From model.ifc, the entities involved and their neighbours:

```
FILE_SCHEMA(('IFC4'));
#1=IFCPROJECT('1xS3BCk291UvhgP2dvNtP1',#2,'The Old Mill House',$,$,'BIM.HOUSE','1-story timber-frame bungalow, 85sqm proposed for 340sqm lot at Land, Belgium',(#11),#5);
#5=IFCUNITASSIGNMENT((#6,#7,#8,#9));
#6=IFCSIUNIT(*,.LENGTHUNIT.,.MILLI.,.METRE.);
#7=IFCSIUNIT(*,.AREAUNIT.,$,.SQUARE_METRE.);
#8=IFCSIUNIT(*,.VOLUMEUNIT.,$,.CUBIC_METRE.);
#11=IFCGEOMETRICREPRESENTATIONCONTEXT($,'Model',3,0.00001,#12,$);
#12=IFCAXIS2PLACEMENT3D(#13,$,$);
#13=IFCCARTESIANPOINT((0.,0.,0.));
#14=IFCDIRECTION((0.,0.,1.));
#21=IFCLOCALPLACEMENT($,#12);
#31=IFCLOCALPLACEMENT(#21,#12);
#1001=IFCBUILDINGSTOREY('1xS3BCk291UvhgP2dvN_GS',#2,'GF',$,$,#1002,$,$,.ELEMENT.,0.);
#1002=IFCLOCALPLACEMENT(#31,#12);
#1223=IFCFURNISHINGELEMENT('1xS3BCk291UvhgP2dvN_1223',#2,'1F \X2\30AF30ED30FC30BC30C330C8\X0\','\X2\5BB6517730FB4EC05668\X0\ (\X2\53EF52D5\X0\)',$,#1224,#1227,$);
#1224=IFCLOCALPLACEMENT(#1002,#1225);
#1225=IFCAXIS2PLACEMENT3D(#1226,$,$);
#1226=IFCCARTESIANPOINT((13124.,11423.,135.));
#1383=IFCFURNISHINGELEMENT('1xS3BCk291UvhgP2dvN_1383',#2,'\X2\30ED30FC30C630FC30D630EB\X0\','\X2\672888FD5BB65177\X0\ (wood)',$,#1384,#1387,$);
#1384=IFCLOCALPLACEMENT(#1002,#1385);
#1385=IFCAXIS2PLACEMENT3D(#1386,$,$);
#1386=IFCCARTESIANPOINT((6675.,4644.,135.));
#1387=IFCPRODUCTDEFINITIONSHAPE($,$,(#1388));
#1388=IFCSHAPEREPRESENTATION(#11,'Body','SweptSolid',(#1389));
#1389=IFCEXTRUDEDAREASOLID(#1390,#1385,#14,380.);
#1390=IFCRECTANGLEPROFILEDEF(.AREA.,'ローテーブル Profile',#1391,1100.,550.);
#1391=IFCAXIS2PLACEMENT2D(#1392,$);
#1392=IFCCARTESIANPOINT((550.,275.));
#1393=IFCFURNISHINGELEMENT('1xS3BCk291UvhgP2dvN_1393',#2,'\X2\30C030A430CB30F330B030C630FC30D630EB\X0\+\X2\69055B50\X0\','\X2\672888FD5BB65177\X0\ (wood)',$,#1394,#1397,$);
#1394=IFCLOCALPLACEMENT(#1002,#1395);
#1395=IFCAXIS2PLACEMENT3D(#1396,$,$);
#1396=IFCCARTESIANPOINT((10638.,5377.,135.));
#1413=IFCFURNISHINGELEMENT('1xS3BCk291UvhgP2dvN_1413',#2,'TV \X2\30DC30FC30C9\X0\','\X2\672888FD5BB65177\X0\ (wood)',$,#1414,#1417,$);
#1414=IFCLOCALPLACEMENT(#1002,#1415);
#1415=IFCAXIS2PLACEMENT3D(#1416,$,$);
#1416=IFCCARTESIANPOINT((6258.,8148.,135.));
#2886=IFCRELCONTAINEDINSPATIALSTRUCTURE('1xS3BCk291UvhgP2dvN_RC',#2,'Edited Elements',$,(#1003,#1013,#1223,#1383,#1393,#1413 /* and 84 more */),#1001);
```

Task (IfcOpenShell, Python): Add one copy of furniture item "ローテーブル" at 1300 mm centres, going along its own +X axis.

```python
import ifcopenshell
import ifcopenshell.api.geometry
import ifcopenshell.api.root
import ifcopenshell.util.element
import ifcopenshell.util.placement

model = ifcopenshell.open("model.ifc")


def reuse_history(source, copy):
    """copy_class also copies each property set's owner history, people and application; keep the originals."""
    for rel in copy.IsDefinedBy:
        if rel.is_a("IfcRelDefinesByProperties") and (history := rel.RelatingPropertyDefinition.OwnerHistory):
            rel.RelatingPropertyDefinition.OwnerHistory = source.OwnerHistory
            ifcopenshell.util.element.remove_deep2(model, history)


source = model.by_guid("1xS3BCk291UvhgP2dvN_1383")
base = ifcopenshell.util.placement.get_local_placement(source.ObjectPlacement)
step = base[:3, 0] * 1300.0

for i in range(1, 2):
    copy = ifcopenshell.api.root.copy_class(model, product=source)
    copy.Representation = ifcopenshell.util.element.copy_deep(
        model, source.Representation, exclude=["IfcGeometricRepresentationContext", "IfcRepresentationMap"]
    )
    reuse_history(source, copy)
    matrix = base.copy()
    matrix[:3, 3] += i * step
    print("added at", matrix[:3, 3].round(3) + 0.0)
    ifcopenshell.api.geometry.edit_object_placement(model, product=copy, matrix=matrix, is_si=False)

model.write("model-out.ifc")
```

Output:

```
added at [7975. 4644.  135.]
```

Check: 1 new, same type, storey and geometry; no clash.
